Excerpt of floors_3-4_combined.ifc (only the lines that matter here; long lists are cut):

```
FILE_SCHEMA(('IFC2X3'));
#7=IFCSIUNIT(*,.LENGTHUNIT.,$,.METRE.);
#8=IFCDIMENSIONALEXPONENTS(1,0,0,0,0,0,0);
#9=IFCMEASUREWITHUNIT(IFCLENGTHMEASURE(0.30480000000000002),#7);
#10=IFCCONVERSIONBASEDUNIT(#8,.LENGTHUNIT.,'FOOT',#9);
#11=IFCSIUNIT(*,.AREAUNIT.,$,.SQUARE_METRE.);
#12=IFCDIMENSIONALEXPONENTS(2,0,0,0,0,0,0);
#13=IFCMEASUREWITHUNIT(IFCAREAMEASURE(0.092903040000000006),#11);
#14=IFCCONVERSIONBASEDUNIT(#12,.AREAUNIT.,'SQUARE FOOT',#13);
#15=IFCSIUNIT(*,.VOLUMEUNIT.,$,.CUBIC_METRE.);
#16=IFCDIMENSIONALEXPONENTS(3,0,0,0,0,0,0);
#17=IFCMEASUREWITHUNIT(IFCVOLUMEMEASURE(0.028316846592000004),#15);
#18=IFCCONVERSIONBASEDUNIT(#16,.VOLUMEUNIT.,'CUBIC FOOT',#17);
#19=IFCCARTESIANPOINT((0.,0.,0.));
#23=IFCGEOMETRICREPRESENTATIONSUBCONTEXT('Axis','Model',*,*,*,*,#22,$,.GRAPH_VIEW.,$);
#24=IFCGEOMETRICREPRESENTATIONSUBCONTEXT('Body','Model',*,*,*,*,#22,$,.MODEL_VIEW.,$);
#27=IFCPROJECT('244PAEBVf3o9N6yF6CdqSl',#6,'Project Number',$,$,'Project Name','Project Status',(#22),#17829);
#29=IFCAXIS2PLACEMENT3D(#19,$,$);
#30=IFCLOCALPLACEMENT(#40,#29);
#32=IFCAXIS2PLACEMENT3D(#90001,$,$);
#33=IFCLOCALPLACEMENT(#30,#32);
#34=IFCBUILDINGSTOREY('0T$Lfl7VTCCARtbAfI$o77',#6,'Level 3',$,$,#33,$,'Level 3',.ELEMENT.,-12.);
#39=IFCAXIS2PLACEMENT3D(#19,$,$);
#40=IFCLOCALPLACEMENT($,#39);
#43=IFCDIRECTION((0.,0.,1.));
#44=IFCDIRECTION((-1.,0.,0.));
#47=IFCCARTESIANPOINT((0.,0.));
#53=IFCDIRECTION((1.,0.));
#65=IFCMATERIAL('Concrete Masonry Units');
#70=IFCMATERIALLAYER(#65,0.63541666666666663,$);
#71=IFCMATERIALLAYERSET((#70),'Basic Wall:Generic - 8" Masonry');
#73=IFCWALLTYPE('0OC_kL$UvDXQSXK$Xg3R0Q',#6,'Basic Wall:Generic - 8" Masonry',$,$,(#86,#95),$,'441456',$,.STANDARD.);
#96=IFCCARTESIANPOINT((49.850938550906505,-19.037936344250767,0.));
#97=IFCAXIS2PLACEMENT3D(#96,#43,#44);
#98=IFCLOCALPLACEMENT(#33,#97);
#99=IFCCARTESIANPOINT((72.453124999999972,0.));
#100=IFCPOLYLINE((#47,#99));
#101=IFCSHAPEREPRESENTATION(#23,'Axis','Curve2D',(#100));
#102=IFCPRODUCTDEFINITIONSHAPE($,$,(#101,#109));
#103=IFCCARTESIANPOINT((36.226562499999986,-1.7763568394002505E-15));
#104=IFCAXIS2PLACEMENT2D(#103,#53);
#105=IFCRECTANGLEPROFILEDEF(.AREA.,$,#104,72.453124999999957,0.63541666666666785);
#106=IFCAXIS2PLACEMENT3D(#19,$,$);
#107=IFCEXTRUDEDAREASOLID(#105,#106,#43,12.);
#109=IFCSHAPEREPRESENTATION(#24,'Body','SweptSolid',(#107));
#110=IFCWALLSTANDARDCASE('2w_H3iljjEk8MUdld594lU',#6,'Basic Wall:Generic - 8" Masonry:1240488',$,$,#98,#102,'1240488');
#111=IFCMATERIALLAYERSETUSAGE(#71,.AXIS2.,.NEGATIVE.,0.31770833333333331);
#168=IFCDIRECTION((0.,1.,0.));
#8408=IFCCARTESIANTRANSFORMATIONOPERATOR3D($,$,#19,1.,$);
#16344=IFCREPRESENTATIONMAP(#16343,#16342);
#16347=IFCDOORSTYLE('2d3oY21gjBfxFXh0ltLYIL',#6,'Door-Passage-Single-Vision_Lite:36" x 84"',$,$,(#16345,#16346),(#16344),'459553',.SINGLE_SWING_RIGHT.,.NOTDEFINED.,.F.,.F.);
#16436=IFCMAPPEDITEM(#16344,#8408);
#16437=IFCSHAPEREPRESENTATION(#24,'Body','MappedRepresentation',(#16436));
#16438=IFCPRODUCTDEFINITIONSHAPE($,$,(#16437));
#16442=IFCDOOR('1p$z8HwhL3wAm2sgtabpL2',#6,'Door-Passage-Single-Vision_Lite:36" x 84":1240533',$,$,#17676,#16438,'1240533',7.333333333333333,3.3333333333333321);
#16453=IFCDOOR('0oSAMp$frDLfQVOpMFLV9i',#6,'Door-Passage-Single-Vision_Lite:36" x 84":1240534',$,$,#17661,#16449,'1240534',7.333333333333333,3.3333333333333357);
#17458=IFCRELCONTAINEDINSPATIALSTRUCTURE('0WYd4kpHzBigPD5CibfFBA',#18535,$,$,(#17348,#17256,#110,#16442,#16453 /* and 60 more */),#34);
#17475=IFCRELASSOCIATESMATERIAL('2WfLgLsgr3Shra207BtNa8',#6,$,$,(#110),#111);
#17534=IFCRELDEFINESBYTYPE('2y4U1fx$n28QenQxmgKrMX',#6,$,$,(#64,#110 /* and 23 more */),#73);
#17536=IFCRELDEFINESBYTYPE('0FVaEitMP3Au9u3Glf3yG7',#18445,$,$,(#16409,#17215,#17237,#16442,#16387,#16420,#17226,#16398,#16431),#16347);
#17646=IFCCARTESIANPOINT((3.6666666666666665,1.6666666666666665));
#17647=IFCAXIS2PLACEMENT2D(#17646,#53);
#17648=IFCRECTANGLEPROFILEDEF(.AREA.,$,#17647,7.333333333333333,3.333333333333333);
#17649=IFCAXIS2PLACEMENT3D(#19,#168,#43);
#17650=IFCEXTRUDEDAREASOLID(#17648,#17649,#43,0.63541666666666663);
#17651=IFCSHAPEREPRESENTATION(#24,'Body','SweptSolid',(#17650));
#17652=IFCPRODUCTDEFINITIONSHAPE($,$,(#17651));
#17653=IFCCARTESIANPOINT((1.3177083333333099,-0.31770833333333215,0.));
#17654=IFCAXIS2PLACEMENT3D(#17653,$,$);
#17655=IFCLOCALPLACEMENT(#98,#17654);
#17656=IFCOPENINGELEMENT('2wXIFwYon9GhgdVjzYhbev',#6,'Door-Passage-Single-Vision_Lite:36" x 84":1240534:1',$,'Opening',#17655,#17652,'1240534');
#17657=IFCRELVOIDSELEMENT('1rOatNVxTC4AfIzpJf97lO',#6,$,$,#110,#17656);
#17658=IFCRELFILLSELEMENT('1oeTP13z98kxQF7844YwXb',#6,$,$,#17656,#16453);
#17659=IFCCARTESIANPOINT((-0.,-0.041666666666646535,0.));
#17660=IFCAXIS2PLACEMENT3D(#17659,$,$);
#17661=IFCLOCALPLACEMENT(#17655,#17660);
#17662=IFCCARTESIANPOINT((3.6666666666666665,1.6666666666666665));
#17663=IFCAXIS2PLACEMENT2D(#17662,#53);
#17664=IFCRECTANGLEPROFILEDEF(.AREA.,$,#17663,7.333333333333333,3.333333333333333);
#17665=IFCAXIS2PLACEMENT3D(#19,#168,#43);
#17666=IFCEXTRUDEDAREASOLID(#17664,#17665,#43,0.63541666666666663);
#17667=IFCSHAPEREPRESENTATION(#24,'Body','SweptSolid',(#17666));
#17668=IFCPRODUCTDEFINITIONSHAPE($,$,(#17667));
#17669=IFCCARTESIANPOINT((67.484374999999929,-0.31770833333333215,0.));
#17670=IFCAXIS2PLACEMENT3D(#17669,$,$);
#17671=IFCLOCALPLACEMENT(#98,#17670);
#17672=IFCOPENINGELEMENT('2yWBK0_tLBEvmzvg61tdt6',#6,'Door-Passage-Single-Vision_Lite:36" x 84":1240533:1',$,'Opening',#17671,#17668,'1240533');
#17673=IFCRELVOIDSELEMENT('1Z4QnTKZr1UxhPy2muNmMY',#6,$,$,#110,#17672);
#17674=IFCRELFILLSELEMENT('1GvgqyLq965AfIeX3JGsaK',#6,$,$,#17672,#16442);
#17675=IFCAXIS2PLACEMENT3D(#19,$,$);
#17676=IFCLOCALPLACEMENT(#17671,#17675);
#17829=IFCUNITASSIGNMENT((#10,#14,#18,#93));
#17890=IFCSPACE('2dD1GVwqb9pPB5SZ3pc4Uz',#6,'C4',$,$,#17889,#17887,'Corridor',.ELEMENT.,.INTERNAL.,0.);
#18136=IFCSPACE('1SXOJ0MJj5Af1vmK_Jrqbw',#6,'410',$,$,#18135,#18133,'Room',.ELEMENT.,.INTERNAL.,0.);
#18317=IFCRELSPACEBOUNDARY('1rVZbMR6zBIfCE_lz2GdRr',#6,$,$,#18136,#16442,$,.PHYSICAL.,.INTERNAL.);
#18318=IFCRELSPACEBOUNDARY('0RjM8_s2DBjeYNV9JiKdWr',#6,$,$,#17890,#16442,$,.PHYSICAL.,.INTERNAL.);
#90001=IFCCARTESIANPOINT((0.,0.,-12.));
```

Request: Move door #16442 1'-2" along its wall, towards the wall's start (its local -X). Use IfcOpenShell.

```python
import ifcopenshell
import ifcopenshell.api.geometry
import ifcopenshell.util.placement
import ifcopenshell.util.unit

model = ifcopenshell.open("floors_3-4_combined.ifc")
unit_scale = ifcopenshell.util.unit.calculate_unit_scale(model)

door = model.by_id(16442)
opening = door.FillsVoids[0].RelatingOpeningElement
wall = opening.VoidsElements[0].RelatingBuildingElement

wall_matrix = ifcopenshell.util.placement.get_local_placement(wall.ObjectPlacement)
shift = wall_matrix[:3, 0] * -14 * 0.0254 / unit_scale
before = ifcopenshell.util.placement.get_local_placement(door.ObjectPlacement)[:3, 3].copy()

# The door is placed relative to its opening, so it follows when the opening moves.
matrix = ifcopenshell.util.placement.get_local_placement(opening.ObjectPlacement)
matrix[:3, 3] += shift
ifcopenshell.api.geometry.edit_object_placement(
    model, product=opening, matrix=matrix, is_si=False, should_transform_children=True
)

after = ifcopenshell.util.placement.get_local_placement(door.ObjectPlacement)[:3, 3]
print("door moved by", (after - before).round(3) + 0.0)

model.write("floors_3-4_combined_edited.ifc")
```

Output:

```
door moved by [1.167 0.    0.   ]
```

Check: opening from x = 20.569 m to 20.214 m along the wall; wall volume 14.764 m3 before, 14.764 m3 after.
